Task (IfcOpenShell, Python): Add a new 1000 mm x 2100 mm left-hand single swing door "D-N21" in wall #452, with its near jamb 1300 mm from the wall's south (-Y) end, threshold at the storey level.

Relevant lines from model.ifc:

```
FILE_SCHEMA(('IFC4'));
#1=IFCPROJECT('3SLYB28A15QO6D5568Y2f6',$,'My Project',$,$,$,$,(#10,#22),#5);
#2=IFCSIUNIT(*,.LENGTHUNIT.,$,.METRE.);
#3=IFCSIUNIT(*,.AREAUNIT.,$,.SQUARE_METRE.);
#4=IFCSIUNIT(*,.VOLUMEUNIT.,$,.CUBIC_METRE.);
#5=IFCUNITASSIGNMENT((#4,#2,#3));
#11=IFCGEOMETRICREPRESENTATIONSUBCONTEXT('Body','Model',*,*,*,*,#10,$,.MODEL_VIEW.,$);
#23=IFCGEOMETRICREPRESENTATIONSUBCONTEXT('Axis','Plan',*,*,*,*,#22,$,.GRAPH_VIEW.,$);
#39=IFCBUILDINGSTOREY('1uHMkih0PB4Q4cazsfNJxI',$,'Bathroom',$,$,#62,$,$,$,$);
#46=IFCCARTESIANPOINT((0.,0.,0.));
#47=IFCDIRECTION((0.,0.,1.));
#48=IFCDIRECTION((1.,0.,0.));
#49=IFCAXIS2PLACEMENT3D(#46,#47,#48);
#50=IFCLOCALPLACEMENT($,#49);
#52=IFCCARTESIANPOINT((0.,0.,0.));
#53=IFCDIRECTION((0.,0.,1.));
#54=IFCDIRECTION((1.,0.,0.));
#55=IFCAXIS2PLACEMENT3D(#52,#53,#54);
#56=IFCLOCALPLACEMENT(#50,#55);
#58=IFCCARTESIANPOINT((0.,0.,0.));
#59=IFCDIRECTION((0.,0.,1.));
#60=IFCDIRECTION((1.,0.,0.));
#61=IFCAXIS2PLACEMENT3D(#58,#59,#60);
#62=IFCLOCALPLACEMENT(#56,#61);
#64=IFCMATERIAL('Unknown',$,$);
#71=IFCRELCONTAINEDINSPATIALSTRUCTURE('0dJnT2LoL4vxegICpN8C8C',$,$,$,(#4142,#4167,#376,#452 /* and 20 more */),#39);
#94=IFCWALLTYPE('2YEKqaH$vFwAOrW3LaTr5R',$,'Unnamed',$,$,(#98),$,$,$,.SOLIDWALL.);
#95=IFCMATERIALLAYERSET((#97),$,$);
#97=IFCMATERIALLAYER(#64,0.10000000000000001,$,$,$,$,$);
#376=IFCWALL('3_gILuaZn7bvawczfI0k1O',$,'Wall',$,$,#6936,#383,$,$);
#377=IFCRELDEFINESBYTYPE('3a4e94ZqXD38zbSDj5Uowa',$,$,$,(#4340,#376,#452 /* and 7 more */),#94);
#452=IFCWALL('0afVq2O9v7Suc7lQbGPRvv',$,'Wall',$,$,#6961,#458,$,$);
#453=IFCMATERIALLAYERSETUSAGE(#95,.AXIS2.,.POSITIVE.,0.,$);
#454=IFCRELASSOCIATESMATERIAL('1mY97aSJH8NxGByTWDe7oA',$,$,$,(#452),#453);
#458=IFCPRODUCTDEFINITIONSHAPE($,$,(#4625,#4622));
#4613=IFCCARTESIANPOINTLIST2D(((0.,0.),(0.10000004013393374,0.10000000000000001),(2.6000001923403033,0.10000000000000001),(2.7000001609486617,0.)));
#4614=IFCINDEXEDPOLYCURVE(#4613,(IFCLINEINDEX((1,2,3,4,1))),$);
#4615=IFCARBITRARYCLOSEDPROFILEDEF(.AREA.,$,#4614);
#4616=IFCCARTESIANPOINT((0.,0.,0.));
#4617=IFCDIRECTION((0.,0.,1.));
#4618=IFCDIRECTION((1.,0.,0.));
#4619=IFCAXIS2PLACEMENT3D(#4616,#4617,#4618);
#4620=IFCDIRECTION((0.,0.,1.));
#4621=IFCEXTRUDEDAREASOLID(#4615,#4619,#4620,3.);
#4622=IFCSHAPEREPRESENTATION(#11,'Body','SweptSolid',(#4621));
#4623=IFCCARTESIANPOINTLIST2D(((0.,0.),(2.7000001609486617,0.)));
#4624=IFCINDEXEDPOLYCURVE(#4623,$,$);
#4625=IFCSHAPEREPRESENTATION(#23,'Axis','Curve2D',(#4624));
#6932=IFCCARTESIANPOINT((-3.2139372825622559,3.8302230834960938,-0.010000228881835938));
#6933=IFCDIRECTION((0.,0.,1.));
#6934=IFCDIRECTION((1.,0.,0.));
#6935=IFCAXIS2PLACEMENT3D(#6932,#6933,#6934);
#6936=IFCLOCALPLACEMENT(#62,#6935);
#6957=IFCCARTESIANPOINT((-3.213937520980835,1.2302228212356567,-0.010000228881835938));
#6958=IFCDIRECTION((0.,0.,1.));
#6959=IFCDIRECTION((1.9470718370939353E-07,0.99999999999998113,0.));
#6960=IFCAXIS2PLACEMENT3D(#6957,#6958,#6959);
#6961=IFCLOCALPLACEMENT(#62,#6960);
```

```python
import numpy as np
import ifcopenshell
import ifcopenshell.api.feature
import ifcopenshell.api.geometry
import ifcopenshell.api.root
import ifcopenshell.api.spatial
import ifcopenshell.geom
import ifcopenshell.util.element
import ifcopenshell.util.placement
import ifcopenshell.util.representation
import ifcopenshell.util.shape
import ifcopenshell.util.unit

model = ifcopenshell.open("model.ifc")
unit_scale = ifcopenshell.util.unit.calculate_unit_scale(model)
settings = ifcopenshell.geom.settings()


def volume(element):
    """Net volume in cubic metres, openings subtracted."""
    shape = ifcopenshell.geom.create_shape(settings, element)
    return ifcopenshell.util.shape.get_volume(shape.geometry)


wall = model.by_guid("0afVq2O9v7Suc7lQbGPRvv")
storey = ifcopenshell.util.element.get_container(wall, ifc_class="IfcBuildingStorey")
context = ifcopenshell.util.representation.get_context(model, "Model", "Body", "MODEL_VIEW")
before = volume(wall)

width, height, from_end, sill = 1, 2.1, 1.3, 0.0  # metres

# The wall runs along its own X axis, and the end named is its -X end.
wall_shape = ifcopenshell.geom.create_shape(settings, wall)
x, y, z = ifcopenshell.util.shape.get_vertices(wall_shape.geometry).T
start = x.min() + from_end
face, thickness = float(y.min()), float(y.max() - y.min())
wall_matrix = ifcopenshell.util.placement.get_local_placement(wall.ObjectPlacement)
level = ifcopenshell.util.placement.get_local_placement(storey.ObjectPlacement)[2, 3]


def in_wall(x, y):
    """Placement at x, y metres in the wall's axes, at sill height."""
    matrix = wall_matrix.copy()
    matrix[:, 3] = wall_matrix @ np.array([x / unit_scale, y / unit_scale, 0.0, 1.0])
    matrix[2, 3] = level + sill / unit_scale
    return matrix


# Opening: a box that overshoots both wall faces by 50 mm.
opening = ifcopenshell.api.root.create_entity(model, ifc_class="IfcOpeningElement", predefined_type="OPENING")
box = ifcopenshell.api.geometry.add_wall_representation(
    model, context=context, length=width, height=height, thickness=thickness + 0.1
)
ifcopenshell.api.geometry.assign_representation(model, product=opening, representation=box)
ifcopenshell.api.geometry.edit_object_placement(model, product=opening, matrix=in_wall(start, face - 0.05), is_si=False)
ifcopenshell.api.feature.add_feature(model, feature=opening, element=wall)

door = ifcopenshell.api.root.create_entity(model, ifc_class="IfcDoor", name="D-N21", predefined_type="DOOR")
door.OverallWidth, door.OverallHeight = width / unit_scale, height / unit_scale
door.OperationType = "SINGLE_SWING_LEFT"
body = ifcopenshell.api.geometry.add_door_representation(
    model,
    context=context,
    overall_width=door.OverallWidth,
    overall_height=door.OverallHeight,
    operation_type="SINGLE_SWING_LEFT",
    lining_properties={"LiningDepth": thickness / unit_scale, "ThresholdDepth": thickness / unit_scale},
)
ifcopenshell.api.geometry.assign_representation(model, product=door, representation=body)
ifcopenshell.api.spatial.assign_container(model, products=[door], relating_structure=storey)
ifcopenshell.api.feature.add_filling(model, opening=opening, element=door)

# The lining spans the wall, so the door starts at the wall face.
ifcopenshell.api.geometry.edit_object_placement(model, product=door, matrix=in_wall(start, face), is_si=False)

after = volume(wall)

print(f"wall volume {before:.3f} -> {after:.3f} m3")

model.write("model_edited.ifc")
```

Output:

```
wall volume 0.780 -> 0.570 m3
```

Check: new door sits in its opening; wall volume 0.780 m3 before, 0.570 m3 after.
